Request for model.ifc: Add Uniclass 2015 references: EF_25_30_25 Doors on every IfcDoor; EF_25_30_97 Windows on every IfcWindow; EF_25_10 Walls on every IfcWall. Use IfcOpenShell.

First a look at what the model holds.

```python
import ifcopenshell

model = ifcopenshell.open("model.ifc")
print(model.schema)
print("classifications:", [c.Name for c in model.by_type("IfcClassification")])
for ifc_class in ("IfcDoor", "IfcRoof", "IfcStair", "IfcWall", "IfcWindow"):
    print(ifc_class, len(model.by_type(ifc_class)))
```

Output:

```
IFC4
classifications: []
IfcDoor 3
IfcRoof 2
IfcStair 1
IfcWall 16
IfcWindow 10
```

```python
import ifcopenshell
import ifcopenshell.api.classification

model = ifcopenshell.open("model.ifc")

system = ifcopenshell.api.classification.add_classification(model, classification="Uniclass 2015")

codes = {
    "IfcDoor": ("EF_25_30_25", "Doors"),
    "IfcWindow": ("EF_25_30_97", "Windows"),
    "IfcWall": ("EF_25_10", "Walls"),
}
for ifc_class, (code, name) in codes.items():
    products = model.by_type(ifc_class)
    ifcopenshell.api.classification.add_reference(
        model, products=products, classification=system, identification=code, name=name
    )
    print(code, len(products))

model.write("model_v2.ifc")
```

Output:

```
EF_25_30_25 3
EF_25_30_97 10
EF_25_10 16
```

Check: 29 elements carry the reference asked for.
